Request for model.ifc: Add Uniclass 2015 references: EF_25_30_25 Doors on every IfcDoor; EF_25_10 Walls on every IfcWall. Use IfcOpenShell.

First a look at what the model holds.

```python
import ifcopenshell

model = ifcopenshell.open("model.ifc")
print(model.schema)
print("classifications:", [c.Name for c in model.by_type("IfcClassification")])
for ifc_class in ("IfcDoor", "IfcRoof", "IfcStair", "IfcWall", "IfcWindow"):
    print(ifc_class, len(model.by_type(ifc_class)))
```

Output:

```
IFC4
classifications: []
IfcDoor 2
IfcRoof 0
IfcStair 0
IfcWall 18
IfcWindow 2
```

```python
import ifcopenshell
import ifcopenshell.api.classification

model = ifcopenshell.open("model.ifc")

system = ifcopenshell.api.classification.add_classification(model, classification="Uniclass 2015")

codes = {
    "IfcDoor": ("EF_25_30_25", "Doors"),
    "IfcWall": ("EF_25_10", "Walls"),
}
for ifc_class, (code, name) in codes.items():
    products = model.by_type(ifc_class)
    ifcopenshell.api.classification.add_reference(
        model, products=products, classification=system, identification=code, name=name
    )
    print(code, len(products))

model.write("model_updated.ifc")
```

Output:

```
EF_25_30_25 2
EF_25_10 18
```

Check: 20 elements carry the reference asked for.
